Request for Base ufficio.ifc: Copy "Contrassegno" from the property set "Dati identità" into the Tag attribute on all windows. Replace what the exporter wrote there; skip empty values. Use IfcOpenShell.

First a look at what the model holds.

```python
import ifcopenshell
import ifcopenshell.util.element

model = ifcopenshell.open("Base ufficio.ifc")
print(model.schema)
windows = model.by_type("IfcWindow")
print(len(windows), "windows")
for e in windows[:8]:
    source = ifcopenshell.util.element.get_pset(e, "Dati identità", "Contrassegno")
    target = e.Tag
    print(e.id(), repr(source), repr(target), sep=" | ")
```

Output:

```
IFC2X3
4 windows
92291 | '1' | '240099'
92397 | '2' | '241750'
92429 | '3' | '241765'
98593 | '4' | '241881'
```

```python
import ifcopenshell
import ifcopenshell.util.element

model = ifcopenshell.open("Base ufficio.ifc")

count = 0
for e in model.by_type("IfcWindow"):
    value = ifcopenshell.util.element.get_pset(e, "Dati identità", "Contrassegno")
    current = e.Tag
    if not value or not value.strip() or current == value:
        continue
    e.Tag = value
    count += 1

print(count, "windows updated")

model.write("Base ufficio_v2.ifc")
```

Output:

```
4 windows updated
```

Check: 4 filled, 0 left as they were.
